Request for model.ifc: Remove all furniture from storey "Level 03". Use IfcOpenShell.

First a look at what the model holds.

```python
import ifcopenshell
import ifcopenshell.util.element

model = ifcopenshell.open("model.ifc")
print(model.schema)
storey = next(s for s in model.by_type("IfcBuildingStorey") if s.Name == "Level 03")
furniture = [e for e in ifcopenshell.util.element.get_decomposition(storey) if e.is_a("IfcFurnishingElement")]
seen = {}
for e in furniture:
    element_type = ifcopenshell.util.element.get_type(e)
    name = element_type.Name if element_type not in (None, e) else None
    seen[name] = seen.get(name, 0) + 1
for name, count in sorted(seen.items(), key=str):
    print(count, "x", name)
```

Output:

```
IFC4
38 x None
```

```python
import ifcopenshell
import ifcopenshell.api.root
import ifcopenshell.util.element

model = ifcopenshell.open("model.ifc")

storey = next(s for s in model.by_type("IfcBuildingStorey") if s.Name == "Level 03")
furniture = [e for e in ifcopenshell.util.element.get_decomposition(storey) if e.is_a("IfcFurnishingElement")]

for e in furniture:
    ifcopenshell.api.root.remove_product(model, product=e)
print(len(furniture), "removed")

model.write("model_v2.ifc")
```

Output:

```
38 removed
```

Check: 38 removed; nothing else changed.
